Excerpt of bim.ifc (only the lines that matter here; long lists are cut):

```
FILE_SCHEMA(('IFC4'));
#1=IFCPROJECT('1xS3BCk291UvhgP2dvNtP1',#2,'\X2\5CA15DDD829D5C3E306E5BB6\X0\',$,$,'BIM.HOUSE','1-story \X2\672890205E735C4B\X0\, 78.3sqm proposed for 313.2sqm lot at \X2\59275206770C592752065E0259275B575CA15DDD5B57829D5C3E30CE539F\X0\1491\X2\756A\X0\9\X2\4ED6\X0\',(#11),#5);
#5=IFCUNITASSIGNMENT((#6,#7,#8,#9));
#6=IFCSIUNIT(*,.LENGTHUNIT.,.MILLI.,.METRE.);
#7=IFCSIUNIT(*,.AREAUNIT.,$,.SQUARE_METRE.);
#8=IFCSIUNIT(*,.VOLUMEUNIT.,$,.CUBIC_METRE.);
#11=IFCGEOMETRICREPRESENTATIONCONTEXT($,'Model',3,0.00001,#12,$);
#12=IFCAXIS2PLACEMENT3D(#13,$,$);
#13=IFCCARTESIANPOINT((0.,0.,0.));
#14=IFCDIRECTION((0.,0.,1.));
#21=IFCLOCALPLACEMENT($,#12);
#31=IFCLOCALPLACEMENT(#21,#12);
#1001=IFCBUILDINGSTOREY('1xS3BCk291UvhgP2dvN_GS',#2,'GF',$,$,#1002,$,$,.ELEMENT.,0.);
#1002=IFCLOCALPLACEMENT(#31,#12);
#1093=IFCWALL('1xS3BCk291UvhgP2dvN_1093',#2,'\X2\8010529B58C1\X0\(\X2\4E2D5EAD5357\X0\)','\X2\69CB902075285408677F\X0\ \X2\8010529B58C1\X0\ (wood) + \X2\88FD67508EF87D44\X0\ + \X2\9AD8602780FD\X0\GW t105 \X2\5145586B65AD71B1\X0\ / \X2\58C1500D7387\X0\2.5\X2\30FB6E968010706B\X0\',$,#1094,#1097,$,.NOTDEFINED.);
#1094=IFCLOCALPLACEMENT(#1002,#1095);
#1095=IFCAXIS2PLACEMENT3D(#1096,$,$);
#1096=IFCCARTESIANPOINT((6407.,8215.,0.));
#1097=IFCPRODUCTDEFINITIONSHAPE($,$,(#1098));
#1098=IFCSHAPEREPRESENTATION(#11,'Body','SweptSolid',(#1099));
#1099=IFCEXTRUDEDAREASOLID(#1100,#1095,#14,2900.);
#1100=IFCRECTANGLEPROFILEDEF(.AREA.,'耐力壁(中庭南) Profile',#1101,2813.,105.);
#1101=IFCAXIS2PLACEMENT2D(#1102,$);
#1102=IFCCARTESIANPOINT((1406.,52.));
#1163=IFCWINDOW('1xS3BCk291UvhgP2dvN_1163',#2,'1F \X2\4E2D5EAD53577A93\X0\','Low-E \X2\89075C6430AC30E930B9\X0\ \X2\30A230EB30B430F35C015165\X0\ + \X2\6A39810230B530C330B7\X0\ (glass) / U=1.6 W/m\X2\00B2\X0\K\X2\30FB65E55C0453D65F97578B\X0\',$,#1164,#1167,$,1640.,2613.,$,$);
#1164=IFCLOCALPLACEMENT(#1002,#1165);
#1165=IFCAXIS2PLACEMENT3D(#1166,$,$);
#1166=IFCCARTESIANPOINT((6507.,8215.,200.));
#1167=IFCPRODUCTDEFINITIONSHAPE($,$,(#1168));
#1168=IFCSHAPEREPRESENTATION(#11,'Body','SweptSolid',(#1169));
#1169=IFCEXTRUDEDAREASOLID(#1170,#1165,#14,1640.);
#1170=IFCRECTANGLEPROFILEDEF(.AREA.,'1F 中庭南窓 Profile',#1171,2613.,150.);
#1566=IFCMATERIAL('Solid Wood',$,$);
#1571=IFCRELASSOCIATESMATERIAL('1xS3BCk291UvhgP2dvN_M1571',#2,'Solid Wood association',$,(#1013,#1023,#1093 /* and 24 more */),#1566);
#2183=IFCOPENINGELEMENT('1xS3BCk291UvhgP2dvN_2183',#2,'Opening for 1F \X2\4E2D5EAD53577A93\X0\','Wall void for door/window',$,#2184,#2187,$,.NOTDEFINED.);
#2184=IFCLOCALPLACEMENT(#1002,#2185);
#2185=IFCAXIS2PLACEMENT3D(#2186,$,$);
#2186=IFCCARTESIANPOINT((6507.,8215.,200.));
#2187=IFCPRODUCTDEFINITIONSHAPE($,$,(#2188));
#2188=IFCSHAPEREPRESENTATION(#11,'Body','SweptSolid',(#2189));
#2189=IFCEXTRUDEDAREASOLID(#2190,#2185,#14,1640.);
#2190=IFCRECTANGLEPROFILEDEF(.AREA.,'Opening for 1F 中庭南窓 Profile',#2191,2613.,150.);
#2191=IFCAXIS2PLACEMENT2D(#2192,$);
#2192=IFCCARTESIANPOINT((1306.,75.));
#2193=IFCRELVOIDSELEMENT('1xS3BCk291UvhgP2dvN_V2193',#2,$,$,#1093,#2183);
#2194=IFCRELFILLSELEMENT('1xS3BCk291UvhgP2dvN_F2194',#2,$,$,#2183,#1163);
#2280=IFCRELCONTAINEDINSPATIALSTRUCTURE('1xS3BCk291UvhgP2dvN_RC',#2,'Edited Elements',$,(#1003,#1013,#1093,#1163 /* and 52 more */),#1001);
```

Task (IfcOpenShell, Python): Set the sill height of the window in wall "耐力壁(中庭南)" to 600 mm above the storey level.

```python
import numpy as np
import ifcopenshell
import ifcopenshell.api.geometry
import ifcopenshell.geom
import ifcopenshell.util.element
import ifcopenshell.util.placement
import ifcopenshell.util.shape
import ifcopenshell.util.unit

model = ifcopenshell.open("bim.ifc")
unit_scale = ifcopenshell.util.unit.calculate_unit_scale(model)

window = model.by_guid("1xS3BCk291UvhgP2dvN_1163")
opening = window.FillsVoids[0].RelatingOpeningElement
storey = ifcopenshell.util.element.get_container(window, ifc_class="IfcBuildingStorey")
level = ifcopenshell.util.placement.get_local_placement(storey.ObjectPlacement)[2, 3]

# The opening's origin need not be at the sill, so measure its lowest point.
shape = ifcopenshell.geom.create_shape(ifcopenshell.geom.settings(), opening)
bottom = ifcopenshell.util.shape.get_shape_bottom_elevation(shape, shape.geometry) / unit_scale
dz = level + 600.0 - bottom

shift = np.array([0.0, 0.0, dz])
# The window is not placed relative to its opening, so move both.
for product in (opening, window):
    matrix = ifcopenshell.util.placement.get_local_placement(product.ObjectPlacement)
    matrix[:3, 3] += shift
    ifcopenshell.api.geometry.edit_object_placement(model, product=product, matrix=matrix, is_si=False)

print(f"moved by {dz * unit_scale:+.3f} m")

model.write("bim_edited.ifc")
```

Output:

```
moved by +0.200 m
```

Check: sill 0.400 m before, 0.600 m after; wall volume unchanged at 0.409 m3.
